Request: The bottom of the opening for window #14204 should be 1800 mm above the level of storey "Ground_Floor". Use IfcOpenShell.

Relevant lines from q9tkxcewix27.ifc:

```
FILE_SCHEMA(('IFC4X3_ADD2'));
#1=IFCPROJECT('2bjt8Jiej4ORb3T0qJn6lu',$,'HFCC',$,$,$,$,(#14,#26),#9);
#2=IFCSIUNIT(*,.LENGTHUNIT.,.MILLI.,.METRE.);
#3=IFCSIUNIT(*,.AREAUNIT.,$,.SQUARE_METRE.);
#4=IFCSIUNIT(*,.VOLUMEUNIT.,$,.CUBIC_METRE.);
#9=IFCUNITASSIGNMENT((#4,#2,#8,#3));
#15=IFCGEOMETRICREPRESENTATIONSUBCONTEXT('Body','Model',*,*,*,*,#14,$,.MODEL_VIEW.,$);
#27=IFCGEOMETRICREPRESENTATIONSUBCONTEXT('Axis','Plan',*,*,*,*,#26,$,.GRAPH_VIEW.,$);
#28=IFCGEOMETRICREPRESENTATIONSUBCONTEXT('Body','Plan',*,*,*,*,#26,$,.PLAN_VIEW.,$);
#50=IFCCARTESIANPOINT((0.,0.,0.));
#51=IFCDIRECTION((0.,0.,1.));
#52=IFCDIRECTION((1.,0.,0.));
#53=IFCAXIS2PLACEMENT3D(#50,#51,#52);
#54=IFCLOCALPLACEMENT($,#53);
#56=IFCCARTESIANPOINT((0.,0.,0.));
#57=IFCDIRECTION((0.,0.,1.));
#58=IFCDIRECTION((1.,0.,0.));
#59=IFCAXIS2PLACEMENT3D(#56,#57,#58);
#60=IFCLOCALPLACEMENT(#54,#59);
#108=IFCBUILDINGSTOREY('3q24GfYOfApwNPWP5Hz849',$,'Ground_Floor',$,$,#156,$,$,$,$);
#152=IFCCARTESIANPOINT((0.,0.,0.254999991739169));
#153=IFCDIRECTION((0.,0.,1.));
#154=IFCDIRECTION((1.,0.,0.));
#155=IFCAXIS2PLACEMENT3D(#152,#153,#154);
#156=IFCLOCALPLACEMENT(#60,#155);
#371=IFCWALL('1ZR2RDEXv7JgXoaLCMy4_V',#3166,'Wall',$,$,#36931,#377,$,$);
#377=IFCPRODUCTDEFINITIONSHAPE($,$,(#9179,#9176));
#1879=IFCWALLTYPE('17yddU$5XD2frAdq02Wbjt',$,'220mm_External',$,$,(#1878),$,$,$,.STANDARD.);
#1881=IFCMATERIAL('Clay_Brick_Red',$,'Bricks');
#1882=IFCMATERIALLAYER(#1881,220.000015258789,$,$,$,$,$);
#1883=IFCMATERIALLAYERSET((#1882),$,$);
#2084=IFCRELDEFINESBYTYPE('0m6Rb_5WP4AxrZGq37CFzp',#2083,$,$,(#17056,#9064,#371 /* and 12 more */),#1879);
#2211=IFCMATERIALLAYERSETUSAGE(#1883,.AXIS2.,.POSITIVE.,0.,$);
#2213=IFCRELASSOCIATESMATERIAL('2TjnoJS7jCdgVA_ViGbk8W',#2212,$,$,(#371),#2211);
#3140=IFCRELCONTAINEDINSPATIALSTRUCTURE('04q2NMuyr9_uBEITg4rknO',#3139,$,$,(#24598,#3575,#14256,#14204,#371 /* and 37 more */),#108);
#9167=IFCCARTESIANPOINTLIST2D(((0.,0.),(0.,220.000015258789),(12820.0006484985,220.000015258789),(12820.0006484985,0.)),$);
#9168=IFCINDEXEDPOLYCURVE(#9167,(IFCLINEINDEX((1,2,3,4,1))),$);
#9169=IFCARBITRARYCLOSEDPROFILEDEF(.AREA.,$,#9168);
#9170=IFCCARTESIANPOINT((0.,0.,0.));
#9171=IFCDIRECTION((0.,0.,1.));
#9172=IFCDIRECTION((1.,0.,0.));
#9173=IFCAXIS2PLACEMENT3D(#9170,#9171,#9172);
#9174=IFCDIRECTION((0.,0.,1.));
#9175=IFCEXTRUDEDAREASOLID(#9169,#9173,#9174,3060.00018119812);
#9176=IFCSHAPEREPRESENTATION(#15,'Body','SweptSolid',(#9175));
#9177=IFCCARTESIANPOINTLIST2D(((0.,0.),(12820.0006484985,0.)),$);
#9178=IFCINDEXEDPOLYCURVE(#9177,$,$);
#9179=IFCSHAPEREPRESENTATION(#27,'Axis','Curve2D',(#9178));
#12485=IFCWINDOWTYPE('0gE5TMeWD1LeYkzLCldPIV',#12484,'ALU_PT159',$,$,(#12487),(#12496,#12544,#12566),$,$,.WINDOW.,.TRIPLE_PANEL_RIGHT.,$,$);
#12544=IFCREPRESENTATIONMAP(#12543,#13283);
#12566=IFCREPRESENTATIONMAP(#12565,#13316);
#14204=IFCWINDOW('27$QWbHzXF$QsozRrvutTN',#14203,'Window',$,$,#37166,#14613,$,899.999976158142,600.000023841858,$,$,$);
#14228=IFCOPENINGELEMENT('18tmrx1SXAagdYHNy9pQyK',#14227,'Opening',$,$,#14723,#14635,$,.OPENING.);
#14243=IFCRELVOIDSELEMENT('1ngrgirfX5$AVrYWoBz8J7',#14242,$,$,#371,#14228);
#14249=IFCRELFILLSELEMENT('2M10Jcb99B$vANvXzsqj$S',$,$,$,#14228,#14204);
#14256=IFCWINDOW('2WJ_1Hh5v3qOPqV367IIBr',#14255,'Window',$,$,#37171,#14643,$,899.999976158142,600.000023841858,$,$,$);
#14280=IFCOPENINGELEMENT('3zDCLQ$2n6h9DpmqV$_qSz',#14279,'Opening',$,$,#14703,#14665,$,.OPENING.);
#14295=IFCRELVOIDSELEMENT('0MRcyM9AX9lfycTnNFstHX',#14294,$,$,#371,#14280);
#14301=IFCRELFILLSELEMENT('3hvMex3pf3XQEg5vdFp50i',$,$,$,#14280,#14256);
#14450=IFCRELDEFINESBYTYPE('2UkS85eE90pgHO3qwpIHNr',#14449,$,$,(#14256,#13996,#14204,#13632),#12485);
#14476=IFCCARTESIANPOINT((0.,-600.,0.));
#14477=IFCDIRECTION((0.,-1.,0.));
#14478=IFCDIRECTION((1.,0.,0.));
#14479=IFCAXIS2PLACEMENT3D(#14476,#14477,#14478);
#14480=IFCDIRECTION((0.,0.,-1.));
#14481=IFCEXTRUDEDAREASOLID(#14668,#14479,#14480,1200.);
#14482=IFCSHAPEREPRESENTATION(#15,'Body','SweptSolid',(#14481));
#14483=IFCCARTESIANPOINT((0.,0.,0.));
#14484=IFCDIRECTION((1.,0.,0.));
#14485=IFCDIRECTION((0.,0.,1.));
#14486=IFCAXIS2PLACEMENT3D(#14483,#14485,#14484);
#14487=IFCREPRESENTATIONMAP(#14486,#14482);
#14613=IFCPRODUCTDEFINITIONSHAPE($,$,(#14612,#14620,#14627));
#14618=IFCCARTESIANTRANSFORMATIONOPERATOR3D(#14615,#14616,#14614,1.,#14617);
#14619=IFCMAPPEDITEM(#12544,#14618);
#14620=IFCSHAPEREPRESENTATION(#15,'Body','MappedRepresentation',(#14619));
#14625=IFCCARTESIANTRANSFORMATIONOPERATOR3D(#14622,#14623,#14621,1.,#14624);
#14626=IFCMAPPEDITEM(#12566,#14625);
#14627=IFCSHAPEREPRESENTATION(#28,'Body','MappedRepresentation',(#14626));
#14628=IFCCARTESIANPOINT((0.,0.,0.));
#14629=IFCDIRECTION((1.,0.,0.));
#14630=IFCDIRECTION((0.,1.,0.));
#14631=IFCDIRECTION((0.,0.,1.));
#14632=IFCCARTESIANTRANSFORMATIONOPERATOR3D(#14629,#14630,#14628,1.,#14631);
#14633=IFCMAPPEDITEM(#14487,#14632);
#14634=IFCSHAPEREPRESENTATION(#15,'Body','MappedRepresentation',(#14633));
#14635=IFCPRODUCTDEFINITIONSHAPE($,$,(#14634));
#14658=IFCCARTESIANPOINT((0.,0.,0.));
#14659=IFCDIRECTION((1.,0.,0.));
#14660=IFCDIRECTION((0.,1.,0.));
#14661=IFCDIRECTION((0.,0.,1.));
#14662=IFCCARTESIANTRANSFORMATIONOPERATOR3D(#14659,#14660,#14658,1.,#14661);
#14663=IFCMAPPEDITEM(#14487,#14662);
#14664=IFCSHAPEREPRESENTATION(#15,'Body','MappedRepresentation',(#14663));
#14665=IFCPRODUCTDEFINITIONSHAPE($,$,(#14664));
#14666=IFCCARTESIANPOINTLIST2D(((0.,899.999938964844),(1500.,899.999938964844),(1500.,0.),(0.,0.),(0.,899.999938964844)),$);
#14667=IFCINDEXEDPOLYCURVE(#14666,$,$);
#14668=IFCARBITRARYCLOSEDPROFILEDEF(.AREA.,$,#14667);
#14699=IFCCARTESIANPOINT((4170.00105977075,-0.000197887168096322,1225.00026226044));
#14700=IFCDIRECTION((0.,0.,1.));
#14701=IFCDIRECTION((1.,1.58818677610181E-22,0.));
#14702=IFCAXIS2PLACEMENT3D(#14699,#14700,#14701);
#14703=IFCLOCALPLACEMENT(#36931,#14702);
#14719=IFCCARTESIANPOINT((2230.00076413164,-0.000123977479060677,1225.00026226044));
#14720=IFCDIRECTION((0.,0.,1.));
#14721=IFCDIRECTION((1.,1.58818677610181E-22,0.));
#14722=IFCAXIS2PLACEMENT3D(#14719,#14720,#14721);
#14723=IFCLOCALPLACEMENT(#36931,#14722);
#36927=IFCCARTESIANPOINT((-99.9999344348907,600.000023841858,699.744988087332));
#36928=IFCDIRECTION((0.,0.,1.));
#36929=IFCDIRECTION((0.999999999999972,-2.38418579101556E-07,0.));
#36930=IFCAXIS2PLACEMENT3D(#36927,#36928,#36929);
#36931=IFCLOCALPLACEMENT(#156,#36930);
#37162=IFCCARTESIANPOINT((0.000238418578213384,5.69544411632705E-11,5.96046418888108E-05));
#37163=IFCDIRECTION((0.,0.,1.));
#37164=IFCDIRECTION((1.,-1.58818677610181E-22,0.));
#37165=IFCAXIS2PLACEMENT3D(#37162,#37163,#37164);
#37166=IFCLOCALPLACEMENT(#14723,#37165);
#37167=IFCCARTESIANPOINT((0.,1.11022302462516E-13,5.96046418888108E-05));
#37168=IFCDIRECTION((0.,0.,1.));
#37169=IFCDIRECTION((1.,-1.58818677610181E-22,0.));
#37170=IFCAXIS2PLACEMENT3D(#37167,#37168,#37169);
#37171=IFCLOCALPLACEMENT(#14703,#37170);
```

```python
import numpy as np
import ifcopenshell
import ifcopenshell.api.geometry
import ifcopenshell.geom
import ifcopenshell.util.element
import ifcopenshell.util.placement
import ifcopenshell.util.shape
import ifcopenshell.util.unit

model = ifcopenshell.open("q9tkxcewix27.ifc")
unit_scale = ifcopenshell.util.unit.calculate_unit_scale(model)

window = model.by_guid("27$QWbHzXF$QsozRrvutTN")
opening = window.FillsVoids[0].RelatingOpeningElement
storey = ifcopenshell.util.element.get_container(window, ifc_class="IfcBuildingStorey")
level = ifcopenshell.util.placement.get_local_placement(storey.ObjectPlacement)[2, 3]

# The opening's origin need not be at the sill, so measure its lowest point.
shape = ifcopenshell.geom.create_shape(ifcopenshell.geom.settings(), opening)
bottom = ifcopenshell.util.shape.get_shape_bottom_elevation(shape, shape.geometry) / unit_scale
dz = level + 1.8 / unit_scale - bottom

shift = np.array([0.0, 0.0, dz])
# The window is placed relative to its opening, so it follows when the opening moves.
matrix = ifcopenshell.util.placement.get_local_placement(opening.ObjectPlacement)
matrix[:3, 3] += shift
ifcopenshell.api.geometry.edit_object_placement(
    model, product=opening, matrix=matrix, is_si=False, should_transform_children=True
)

print(f"moved by {dz * unit_scale:+.3f} m")

model.write("q9tkxcewix27_v2.ifc")
```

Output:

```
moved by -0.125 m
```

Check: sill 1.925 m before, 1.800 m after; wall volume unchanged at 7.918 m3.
